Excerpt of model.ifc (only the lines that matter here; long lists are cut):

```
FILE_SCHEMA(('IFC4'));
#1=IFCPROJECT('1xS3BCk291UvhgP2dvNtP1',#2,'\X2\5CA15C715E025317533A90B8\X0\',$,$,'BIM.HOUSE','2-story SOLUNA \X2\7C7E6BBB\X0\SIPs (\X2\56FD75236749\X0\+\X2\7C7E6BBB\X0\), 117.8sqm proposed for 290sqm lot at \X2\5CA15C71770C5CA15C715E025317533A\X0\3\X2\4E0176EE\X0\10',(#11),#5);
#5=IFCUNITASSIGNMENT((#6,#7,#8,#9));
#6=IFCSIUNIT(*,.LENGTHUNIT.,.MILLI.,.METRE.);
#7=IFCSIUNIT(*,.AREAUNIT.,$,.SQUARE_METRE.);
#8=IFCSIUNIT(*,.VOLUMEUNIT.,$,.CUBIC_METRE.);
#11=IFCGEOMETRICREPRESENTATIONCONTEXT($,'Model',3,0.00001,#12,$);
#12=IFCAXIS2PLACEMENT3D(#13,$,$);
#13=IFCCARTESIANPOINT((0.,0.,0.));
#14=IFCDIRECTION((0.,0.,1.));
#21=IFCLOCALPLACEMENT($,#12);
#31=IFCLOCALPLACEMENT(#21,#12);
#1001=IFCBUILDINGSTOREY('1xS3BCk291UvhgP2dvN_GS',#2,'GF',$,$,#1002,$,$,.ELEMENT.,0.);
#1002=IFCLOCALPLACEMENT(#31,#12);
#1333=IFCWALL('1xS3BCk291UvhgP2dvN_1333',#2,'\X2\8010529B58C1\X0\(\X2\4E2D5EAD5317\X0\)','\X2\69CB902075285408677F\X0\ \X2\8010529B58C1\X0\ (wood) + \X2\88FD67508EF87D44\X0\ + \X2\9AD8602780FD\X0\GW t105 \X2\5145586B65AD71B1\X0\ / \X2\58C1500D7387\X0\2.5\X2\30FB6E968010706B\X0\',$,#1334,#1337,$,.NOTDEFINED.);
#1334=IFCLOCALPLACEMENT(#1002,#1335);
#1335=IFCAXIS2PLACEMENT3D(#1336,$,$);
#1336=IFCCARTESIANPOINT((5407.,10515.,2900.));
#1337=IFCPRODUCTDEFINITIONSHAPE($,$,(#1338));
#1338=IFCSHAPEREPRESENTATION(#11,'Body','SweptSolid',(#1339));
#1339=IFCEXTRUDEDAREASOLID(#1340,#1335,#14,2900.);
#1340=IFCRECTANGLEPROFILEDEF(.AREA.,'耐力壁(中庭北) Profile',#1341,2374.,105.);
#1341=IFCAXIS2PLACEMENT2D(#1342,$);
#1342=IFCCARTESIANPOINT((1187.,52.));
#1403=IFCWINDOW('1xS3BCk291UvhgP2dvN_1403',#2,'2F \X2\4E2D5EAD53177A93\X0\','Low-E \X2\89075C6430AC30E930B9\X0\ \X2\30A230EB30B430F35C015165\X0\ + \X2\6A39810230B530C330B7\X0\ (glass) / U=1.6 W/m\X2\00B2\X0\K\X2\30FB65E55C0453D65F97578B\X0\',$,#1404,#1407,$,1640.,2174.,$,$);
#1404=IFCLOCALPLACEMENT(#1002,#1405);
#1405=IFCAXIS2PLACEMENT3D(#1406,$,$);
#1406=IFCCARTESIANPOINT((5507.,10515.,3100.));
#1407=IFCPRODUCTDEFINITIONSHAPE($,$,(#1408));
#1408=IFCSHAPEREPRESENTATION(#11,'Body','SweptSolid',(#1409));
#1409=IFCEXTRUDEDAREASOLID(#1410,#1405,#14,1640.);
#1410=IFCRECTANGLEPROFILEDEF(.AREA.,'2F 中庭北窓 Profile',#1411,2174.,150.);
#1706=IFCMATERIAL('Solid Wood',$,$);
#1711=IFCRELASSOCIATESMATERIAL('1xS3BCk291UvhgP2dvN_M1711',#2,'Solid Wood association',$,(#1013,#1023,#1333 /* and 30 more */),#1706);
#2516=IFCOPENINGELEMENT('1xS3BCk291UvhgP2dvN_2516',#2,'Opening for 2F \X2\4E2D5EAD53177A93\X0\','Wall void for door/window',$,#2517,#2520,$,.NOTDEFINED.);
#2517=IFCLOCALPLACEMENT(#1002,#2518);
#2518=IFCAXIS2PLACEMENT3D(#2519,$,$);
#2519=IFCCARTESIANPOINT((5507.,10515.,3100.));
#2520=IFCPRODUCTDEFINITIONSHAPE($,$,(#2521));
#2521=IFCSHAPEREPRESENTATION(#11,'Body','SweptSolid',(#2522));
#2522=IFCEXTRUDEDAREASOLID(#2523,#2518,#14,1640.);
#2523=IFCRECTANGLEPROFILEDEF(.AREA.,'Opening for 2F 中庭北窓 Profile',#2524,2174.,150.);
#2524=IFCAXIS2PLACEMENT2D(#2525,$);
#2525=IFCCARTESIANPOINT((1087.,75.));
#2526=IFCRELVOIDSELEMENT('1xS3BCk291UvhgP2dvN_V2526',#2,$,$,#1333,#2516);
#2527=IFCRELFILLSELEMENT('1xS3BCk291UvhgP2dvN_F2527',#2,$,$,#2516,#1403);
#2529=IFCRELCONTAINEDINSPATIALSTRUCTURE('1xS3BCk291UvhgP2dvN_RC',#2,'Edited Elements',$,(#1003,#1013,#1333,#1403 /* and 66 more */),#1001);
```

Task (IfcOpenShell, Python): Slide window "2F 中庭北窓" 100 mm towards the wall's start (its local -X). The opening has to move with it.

```python
import ifcopenshell
import ifcopenshell.api.geometry
import ifcopenshell.util.placement
import ifcopenshell.util.unit

model = ifcopenshell.open("model.ifc")
unit_scale = ifcopenshell.util.unit.calculate_unit_scale(model)

window = model.by_guid("1xS3BCk291UvhgP2dvN_1403")
opening = window.FillsVoids[0].RelatingOpeningElement
wall = opening.VoidsElements[0].RelatingBuildingElement

wall_matrix = ifcopenshell.util.placement.get_local_placement(wall.ObjectPlacement)
shift = wall_matrix[:3, 0] * -0.1 / unit_scale
before = ifcopenshell.util.placement.get_local_placement(window.ObjectPlacement)[:3, 3].copy()

# The window is not placed relative to its opening, so move both.
for product in (opening, window):
    matrix = ifcopenshell.util.placement.get_local_placement(product.ObjectPlacement)
    matrix[:3, 3] += shift
    ifcopenshell.api.geometry.edit_object_placement(model, product=product, matrix=matrix, is_si=False)

after = ifcopenshell.util.placement.get_local_placement(window.ObjectPlacement)[:3, 3]
print("window moved by", (after - before).round(3) + 0.0)

model.write("model_updated.ifc")
```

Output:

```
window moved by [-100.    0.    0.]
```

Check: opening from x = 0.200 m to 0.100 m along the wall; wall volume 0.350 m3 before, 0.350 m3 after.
